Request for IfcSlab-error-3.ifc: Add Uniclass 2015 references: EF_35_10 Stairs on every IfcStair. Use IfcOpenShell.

First a look at what the model holds.

```python
import ifcopenshell

model = ifcopenshell.open("IfcSlab-error-3.ifc")
print(model.schema)
print("classifications:", [c.Name for c in model.by_type("IfcClassification")])
for ifc_class in ("IfcDoor", "IfcRoof", "IfcStair", "IfcWall", "IfcWindow"):
    print(ifc_class, len(model.by_type(ifc_class)))
```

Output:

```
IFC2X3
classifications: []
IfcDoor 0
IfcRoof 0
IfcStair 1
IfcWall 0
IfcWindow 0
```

```python
import ifcopenshell
import ifcopenshell.api.classification

model = ifcopenshell.open("IfcSlab-error-3.ifc")

# IFC2X3 requires Source and Edition and has no link from the project to the system.
system = model.create_entity("IfcClassification", Source="NBS", Edition="2015", Name="Uniclass 2015")

codes = {
    "IfcStair": ("EF_35_10", "Stairs"),
}
for ifc_class, (code, name) in codes.items():
    products = model.by_type(ifc_class)
    ifcopenshell.api.classification.add_reference(
        model, products=products, classification=system, identification=code, name=name
    )
    print(code, len(products))

model.write("IfcSlab-error-3_edited.ifc")
```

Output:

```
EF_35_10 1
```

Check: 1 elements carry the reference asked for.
